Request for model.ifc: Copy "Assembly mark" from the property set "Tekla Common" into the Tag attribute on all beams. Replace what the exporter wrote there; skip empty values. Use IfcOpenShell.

First a look at what the model holds.

```python
import ifcopenshell
import ifcopenshell.util.element

model = ifcopenshell.open("model.ifc")
print(model.schema)
beams = model.by_type("IfcBeam")
print(len(beams), "beams")
for e in beams[:8]:
    source = ifcopenshell.util.element.get_pset(e, "Tekla Common", "Assembly mark")
    target = e.Tag
    print(e.id(), repr(source), repr(target), sep=" | ")
```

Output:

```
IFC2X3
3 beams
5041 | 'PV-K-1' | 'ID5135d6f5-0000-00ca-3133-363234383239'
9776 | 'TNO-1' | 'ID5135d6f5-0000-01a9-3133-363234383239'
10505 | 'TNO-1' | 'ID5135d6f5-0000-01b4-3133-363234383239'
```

```python
import ifcopenshell
import ifcopenshell.util.element

model = ifcopenshell.open("model.ifc")

count = 0
for e in model.by_type("IfcBeam"):
    value = ifcopenshell.util.element.get_pset(e, "Tekla Common", "Assembly mark")
    current = e.Tag
    if not value or not value.strip() or current == value:
        continue
    e.Tag = value
    count += 1

print(count, "beams updated")

model.write("model_v2.ifc")
```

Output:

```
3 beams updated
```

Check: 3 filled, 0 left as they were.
